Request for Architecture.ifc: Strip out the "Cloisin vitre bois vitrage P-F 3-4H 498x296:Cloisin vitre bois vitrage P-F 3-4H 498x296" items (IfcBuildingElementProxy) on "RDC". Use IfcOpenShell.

First a look at what the model holds.

```python
import ifcopenshell
import ifcopenshell.util.element

model = ifcopenshell.open("Architecture.ifc")
print(model.schema)
storey = next(s for s in model.by_type("IfcBuildingStorey") if s.Name == "RDC")
proxies = [e for e in ifcopenshell.util.element.get_decomposition(storey) if e.is_a("IfcBuildingElementProxy")]
seen = {}
for e in proxies:
    element_type = ifcopenshell.util.element.get_type(e)
    name = element_type.Name if element_type not in (None, e) else None
    seen[name] = seen.get(name, 0) + 1
for name, count in sorted(seen.items(), key=str):
    print(count, "x", name)
```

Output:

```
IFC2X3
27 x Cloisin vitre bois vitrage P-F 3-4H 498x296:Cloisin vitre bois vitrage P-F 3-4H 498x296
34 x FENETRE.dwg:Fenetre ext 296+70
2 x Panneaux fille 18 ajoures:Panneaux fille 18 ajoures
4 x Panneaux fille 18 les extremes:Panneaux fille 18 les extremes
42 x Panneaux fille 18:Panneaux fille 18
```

```python
import ifcopenshell
import ifcopenshell.api.root
import ifcopenshell.util.element

model = ifcopenshell.open("Architecture.ifc")

storey = next(s for s in model.by_type("IfcBuildingStorey") if s.Name == "RDC")
proxies = [e for e in ifcopenshell.util.element.get_decomposition(storey) if e.is_a("IfcBuildingElementProxy")]
targets = [e for e in proxies if (t := ifcopenshell.util.element.get_type(e)) not in (None, e) and t.Name == "Cloisin vitre bois vitrage P-F 3-4H 498x296:Cloisin vitre bois vitrage P-F 3-4H 498x296"]

for e in targets:
    ifcopenshell.api.root.remove_product(model, product=e)
print(len(targets), "removed")

model.write("Architecture_rev.ifc")
```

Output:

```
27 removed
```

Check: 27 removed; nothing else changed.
